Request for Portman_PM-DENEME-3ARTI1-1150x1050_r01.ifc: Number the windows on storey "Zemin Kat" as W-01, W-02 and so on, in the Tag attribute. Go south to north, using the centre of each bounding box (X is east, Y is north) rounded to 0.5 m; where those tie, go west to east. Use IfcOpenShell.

First a look at what the model holds.

```python
import ifcopenshell
import ifcopenshell.util.element
import ifcopenshell.util.placement

model = ifcopenshell.open("Portman_PM-DENEME-3ARTI1-1150x1050_r01.ifc")
print(model.schema)
storey = next(s for s in model.by_type("IfcBuildingStorey") if s.Name == "Zemin Kat")
windows = [e for e in ifcopenshell.util.element.get_decomposition(storey) if e.is_a("IfcWindow")]
for e in sorted(windows, key=lambda e: e.id()):
    origin = ifcopenshell.util.placement.get_local_placement(e.ObjectPlacement)[:3, 3]
    print(e.id(), e.Tag, e.Name, origin.round(2) + 0.0, sep=" | ")
```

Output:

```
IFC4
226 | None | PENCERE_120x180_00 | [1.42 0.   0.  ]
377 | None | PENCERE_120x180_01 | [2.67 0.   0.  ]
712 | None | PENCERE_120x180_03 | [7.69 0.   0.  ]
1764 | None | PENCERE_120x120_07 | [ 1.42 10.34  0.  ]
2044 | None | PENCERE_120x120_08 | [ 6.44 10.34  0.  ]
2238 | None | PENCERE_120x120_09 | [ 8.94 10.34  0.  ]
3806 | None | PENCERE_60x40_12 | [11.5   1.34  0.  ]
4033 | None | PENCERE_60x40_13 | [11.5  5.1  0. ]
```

```python
import ifcopenshell
import ifcopenshell.geom
import ifcopenshell.util.element
import ifcopenshell.util.shape

model = ifcopenshell.open("Portman_PM-DENEME-3ARTI1-1150x1050_r01.ifc")
settings = ifcopenshell.geom.settings()
settings.set("use-world-coords", True)


def centre(element):
    shape = ifcopenshell.geom.create_shape(settings, element)
    return ifcopenshell.util.shape.get_bbox_centroid(shape.geometry)


storey = next(s for s in model.by_type("IfcBuildingStorey") if s.Name == "Zemin Kat")
windows = [e for e in ifcopenshell.util.element.get_decomposition(storey) if e.is_a("IfcWindow")]

# Insertion points can sit at a corner or the storey origin, so sort by the geometry (in metres).
centres = {e: centre(e) for e in windows}
windows.sort(key=lambda e: (round(centres[e][1] / 0.5), centres[e][0]))

for i, e in enumerate(windows, start=1):
    number = f"W-{i:02d}"
    e.Tag = number
    print(e.id(), number)

model.write("Portman_PM-DENEME-3ARTI1-1150x1050_r01_updated.ifc")
```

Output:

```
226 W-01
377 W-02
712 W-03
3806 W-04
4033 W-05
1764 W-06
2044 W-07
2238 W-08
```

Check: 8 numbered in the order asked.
